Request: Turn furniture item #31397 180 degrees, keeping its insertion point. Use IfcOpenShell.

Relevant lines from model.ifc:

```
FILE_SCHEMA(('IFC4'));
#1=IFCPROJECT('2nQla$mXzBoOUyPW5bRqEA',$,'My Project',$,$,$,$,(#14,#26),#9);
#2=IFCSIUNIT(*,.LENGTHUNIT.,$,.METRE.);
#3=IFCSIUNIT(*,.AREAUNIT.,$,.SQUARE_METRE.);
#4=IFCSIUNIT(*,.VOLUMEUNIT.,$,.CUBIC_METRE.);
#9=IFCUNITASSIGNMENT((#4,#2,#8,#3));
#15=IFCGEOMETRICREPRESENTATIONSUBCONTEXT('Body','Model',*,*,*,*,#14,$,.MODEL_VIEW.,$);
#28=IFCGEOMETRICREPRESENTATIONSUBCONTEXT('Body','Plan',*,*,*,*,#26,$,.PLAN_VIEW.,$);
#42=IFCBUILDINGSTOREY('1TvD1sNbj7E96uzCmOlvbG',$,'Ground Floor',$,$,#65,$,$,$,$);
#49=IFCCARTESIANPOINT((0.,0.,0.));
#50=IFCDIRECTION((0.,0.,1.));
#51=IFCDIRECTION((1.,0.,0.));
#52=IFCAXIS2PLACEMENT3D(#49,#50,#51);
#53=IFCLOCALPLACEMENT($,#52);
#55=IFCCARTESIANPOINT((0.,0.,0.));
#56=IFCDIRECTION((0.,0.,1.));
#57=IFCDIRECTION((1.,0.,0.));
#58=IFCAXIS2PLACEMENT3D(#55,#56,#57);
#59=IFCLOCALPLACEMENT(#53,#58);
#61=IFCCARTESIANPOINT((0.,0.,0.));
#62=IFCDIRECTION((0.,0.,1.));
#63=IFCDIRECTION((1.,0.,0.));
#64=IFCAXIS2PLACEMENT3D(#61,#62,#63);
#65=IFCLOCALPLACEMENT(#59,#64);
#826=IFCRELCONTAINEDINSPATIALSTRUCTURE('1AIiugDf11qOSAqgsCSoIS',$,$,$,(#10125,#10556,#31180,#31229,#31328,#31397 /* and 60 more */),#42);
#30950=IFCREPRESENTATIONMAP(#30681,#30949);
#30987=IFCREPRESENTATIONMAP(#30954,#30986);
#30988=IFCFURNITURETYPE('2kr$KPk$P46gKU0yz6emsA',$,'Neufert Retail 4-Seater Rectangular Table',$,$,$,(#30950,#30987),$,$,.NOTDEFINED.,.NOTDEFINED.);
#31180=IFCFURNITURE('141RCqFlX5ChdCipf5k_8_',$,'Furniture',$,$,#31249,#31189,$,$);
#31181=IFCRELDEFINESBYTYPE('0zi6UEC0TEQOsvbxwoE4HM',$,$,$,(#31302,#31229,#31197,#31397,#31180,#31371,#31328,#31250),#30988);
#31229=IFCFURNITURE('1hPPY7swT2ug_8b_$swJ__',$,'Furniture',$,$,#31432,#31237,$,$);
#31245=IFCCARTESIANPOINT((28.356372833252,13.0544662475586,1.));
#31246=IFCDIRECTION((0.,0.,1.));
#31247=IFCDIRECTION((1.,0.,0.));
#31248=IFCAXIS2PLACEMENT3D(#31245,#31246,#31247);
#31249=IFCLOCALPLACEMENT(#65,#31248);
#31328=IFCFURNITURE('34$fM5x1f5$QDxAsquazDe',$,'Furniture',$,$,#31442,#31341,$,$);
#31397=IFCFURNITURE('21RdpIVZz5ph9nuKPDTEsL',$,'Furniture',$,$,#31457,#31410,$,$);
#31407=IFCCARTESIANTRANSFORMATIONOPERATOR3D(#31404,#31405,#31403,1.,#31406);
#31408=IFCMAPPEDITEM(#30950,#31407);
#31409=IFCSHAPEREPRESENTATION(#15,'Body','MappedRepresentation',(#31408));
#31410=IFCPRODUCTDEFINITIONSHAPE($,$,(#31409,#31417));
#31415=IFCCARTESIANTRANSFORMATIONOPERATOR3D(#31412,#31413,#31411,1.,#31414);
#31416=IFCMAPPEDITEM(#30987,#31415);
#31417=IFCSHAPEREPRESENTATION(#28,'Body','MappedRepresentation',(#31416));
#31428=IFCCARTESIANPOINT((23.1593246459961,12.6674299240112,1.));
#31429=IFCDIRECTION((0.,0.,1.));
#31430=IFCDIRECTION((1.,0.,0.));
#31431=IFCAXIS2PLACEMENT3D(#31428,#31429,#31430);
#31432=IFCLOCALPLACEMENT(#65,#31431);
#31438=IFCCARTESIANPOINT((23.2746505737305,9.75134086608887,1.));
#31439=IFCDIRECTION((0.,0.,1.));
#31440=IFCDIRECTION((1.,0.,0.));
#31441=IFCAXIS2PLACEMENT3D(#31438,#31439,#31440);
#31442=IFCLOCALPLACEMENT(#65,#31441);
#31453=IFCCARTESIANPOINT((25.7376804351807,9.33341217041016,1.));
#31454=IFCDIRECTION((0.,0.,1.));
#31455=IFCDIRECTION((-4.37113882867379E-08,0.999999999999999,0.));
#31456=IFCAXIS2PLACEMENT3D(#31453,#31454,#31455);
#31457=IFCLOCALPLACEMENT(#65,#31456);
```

```python
import ifcopenshell
import ifcopenshell.api.geometry
import ifcopenshell.util.placement

model = ifcopenshell.open("model.ifc")

item = model.by_guid("21RdpIVZz5ph9nuKPDTEsL")
matrix = ifcopenshell.util.placement.get_local_placement(item.ObjectPlacement)
matrix = matrix @ ifcopenshell.util.placement.rotation(180, "Z")
ifcopenshell.api.geometry.edit_object_placement(model, product=item, matrix=matrix, is_si=False)

print(ifcopenshell.util.placement.get_local_placement(item.ObjectPlacement).round(3) + 0.0)

model.write("model_rev.ifc")
```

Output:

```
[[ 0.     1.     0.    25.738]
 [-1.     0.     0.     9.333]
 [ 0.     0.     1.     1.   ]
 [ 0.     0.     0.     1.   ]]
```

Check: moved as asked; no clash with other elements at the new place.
